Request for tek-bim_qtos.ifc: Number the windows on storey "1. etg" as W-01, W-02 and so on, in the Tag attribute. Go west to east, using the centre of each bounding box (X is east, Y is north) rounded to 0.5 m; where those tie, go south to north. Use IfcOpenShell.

First a look at what the model holds.

```python
import ifcopenshell
import ifcopenshell.util.element
import ifcopenshell.util.placement

model = ifcopenshell.open("tek-bim_qtos.ifc")
print(model.schema)
storey = next(s for s in model.by_type("IfcBuildingStorey") if s.Name == "1. etg")
windows = [e for e in ifcopenshell.util.element.get_decomposition(storey) if e.is_a("IfcWindow")]
for e in sorted(windows, key=lambda e: e.id()):
    origin = ifcopenshell.util.placement.get_local_placement(e.ObjectPlacement)[:3, 3]
    print(e.id(), e.Tag, e.Name, origin.round(2) + 0.0, sep=" | ")
```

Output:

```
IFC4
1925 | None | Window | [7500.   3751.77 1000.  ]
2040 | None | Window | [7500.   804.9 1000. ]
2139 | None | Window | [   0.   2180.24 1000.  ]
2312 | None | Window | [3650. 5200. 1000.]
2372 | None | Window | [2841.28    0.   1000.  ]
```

```python
import ifcopenshell
import ifcopenshell.geom
import ifcopenshell.util.element
import ifcopenshell.util.shape

model = ifcopenshell.open("tek-bim_qtos.ifc")
settings = ifcopenshell.geom.settings()
settings.set("use-world-coords", True)


def centre(element):
    shape = ifcopenshell.geom.create_shape(settings, element)
    return ifcopenshell.util.shape.get_bbox_centroid(shape.geometry)


storey = next(s for s in model.by_type("IfcBuildingStorey") if s.Name == "1. etg")
windows = [e for e in ifcopenshell.util.element.get_decomposition(storey) if e.is_a("IfcWindow")]

# Insertion points can sit at a corner or the storey origin, so sort by the geometry (in metres).
centres = {e: centre(e) for e in windows}
windows.sort(key=lambda e: (round(centres[e][0] / 0.5), centres[e][1]))

for i, e in enumerate(windows, start=1):
    number = f"W-{i:02d}"
    e.Tag = number
    print(e.id(), number)

model.write("tek-bim_qtos_edited.ifc")
```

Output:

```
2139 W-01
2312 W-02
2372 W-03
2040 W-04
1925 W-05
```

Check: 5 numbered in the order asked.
